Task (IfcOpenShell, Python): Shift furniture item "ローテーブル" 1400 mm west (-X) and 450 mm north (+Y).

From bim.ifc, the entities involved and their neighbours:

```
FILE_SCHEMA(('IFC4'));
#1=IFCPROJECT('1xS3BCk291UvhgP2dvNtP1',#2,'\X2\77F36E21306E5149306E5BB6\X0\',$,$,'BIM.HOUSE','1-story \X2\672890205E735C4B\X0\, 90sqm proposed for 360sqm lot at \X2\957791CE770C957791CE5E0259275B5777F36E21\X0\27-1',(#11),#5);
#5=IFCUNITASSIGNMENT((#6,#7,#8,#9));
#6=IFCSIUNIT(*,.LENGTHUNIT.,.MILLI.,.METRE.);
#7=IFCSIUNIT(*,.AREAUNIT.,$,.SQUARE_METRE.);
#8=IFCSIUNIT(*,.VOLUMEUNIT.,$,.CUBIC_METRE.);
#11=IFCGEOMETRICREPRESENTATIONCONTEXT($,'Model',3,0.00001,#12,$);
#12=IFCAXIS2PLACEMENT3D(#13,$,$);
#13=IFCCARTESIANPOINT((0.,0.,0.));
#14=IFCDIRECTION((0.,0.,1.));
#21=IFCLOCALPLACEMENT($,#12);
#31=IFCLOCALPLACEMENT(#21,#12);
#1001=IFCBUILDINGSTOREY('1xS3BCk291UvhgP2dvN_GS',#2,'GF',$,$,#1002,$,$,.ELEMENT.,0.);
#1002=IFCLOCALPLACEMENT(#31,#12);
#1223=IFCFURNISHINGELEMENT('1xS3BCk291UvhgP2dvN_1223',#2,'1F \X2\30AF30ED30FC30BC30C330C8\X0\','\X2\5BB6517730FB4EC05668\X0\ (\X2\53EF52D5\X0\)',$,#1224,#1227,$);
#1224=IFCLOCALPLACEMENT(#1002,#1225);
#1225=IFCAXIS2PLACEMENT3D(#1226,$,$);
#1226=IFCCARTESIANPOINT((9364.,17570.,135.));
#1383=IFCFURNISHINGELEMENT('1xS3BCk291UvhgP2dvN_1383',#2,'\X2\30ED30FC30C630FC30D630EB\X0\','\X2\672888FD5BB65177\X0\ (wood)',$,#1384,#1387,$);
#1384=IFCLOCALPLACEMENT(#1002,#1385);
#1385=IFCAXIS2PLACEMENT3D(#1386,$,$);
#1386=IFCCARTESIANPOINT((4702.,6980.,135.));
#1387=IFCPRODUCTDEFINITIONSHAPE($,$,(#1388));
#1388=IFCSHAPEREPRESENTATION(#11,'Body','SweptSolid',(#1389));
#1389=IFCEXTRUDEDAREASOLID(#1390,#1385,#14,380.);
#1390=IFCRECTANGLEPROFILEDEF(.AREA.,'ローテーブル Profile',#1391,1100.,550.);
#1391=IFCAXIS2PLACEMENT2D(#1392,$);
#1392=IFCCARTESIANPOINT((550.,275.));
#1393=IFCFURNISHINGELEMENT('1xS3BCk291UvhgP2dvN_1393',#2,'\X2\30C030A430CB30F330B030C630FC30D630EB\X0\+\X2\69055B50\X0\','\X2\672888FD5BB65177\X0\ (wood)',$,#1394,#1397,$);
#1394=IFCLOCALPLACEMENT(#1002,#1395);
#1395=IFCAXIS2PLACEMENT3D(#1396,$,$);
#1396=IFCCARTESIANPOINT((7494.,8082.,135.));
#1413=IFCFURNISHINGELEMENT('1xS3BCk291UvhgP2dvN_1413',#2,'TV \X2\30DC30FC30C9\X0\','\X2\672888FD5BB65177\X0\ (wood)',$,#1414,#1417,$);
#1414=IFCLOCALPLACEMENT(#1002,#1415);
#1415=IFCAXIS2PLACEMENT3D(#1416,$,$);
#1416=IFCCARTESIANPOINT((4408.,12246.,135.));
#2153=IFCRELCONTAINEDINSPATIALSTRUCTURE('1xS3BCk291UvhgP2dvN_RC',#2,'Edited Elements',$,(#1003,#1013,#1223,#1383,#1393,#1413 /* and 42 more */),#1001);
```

```python
import ifcopenshell
import ifcopenshell.api.geometry
import ifcopenshell.util.placement
import ifcopenshell.util.unit

model = ifcopenshell.open("bim.ifc")
unit_scale = ifcopenshell.util.unit.calculate_unit_scale(model)

item = model.by_id(1383)
matrix = ifcopenshell.util.placement.get_local_placement(item.ObjectPlacement)
matrix[0, 3] -= 1.4 / unit_scale
matrix[1, 3] += 0.45 / unit_scale
ifcopenshell.api.geometry.edit_object_placement(model, product=item, matrix=matrix, is_si=False)

print(ifcopenshell.util.placement.get_local_placement(item.ObjectPlacement).round(3) + 0.0)

model.write("bim_rev.ifc")
```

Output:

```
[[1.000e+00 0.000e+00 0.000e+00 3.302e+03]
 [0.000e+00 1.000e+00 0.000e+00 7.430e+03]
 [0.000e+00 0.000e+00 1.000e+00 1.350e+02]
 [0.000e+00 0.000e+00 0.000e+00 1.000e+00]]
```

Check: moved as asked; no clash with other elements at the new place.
